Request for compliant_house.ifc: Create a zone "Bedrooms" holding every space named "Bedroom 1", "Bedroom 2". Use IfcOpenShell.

First a look at what the model holds.

```python
import ifcopenshell

model = ifcopenshell.open("compliant_house.ifc")
print(model.schema)
seen = {}
for space in model.by_type("IfcSpace"):
    seen[space.LongName] = seen.get(space.LongName, 0) + 1
for name, count in sorted(seen.items(), key=str):
    print(count, "x", name)
print("zones:", [z.Name for z in model.by_type("IfcZone")][:20])
```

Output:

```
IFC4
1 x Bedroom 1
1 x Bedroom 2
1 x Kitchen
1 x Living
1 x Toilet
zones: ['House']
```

```python
import ifcopenshell
import ifcopenshell.api.group
import ifcopenshell.api.root

model = ifcopenshell.open("compliant_house.ifc")

names = {"Bedroom 1", "Bedroom 2"}
spaces = [s for s in model.by_type("IfcSpace") if s.LongName in names]

zone = ifcopenshell.api.root.create_entity(model, ifc_class="IfcZone", name="Bedrooms")
ifcopenshell.api.group.assign_group(model, products=spaces, group=zone)
print(len(spaces), "spaces in", zone.Name)

model.write("compliant_house_rev.ifc")
```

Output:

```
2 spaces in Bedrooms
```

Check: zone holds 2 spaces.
